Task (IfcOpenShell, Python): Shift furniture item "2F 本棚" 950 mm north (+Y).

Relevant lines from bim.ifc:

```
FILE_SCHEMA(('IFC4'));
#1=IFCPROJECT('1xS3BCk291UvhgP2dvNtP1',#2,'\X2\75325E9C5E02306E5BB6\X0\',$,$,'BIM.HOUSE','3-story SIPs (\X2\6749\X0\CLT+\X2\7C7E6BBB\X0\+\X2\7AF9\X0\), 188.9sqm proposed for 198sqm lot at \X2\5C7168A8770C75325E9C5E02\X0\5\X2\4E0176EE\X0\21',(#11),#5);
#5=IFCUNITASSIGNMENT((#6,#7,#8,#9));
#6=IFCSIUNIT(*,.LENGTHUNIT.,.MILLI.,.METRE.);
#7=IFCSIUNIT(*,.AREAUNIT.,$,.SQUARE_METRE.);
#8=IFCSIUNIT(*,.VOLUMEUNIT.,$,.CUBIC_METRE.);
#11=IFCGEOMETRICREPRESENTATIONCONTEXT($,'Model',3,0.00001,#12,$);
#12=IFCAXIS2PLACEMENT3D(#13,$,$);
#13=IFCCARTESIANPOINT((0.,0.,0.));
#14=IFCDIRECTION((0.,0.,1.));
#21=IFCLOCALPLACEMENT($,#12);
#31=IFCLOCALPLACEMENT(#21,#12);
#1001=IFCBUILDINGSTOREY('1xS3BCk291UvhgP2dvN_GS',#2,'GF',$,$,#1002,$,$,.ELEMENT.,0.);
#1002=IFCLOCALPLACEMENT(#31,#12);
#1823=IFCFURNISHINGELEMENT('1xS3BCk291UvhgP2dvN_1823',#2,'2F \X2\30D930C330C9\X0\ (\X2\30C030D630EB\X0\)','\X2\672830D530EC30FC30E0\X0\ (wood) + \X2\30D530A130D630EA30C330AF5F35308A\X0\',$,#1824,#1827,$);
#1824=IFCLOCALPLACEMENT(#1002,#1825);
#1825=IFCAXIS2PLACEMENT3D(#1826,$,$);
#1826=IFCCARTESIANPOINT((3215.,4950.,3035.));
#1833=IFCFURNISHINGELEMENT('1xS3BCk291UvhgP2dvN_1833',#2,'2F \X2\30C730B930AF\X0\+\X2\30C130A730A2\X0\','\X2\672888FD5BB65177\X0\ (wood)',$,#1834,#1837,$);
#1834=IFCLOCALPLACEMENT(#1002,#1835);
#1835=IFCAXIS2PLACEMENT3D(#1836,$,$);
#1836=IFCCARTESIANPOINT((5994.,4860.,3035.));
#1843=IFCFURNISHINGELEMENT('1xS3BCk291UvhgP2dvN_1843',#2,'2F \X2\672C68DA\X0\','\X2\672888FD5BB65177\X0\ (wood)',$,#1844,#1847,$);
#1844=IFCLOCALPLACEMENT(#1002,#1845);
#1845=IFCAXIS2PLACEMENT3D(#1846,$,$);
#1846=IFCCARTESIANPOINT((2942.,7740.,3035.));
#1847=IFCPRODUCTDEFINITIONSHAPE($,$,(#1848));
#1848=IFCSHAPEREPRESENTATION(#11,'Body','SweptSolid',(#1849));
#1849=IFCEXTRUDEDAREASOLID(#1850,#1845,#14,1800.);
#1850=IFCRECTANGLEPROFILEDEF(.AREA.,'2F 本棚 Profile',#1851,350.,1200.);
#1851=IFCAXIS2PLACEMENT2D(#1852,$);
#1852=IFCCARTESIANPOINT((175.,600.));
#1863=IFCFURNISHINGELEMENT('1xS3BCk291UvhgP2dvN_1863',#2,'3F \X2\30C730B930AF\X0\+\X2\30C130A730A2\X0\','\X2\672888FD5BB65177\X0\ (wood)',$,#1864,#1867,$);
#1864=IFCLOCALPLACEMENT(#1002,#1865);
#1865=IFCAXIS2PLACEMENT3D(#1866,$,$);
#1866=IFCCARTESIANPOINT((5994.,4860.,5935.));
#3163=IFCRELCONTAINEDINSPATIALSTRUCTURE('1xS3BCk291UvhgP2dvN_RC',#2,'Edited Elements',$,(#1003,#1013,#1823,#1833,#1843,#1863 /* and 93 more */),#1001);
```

```python
import ifcopenshell
import ifcopenshell.api.geometry
import ifcopenshell.util.placement
import ifcopenshell.util.unit

model = ifcopenshell.open("bim.ifc")
unit_scale = ifcopenshell.util.unit.calculate_unit_scale(model)

item = model.by_guid("1xS3BCk291UvhgP2dvN_1843")
matrix = ifcopenshell.util.placement.get_local_placement(item.ObjectPlacement)
matrix[1, 3] += 0.95 / unit_scale
ifcopenshell.api.geometry.edit_object_placement(model, product=item, matrix=matrix, is_si=False)

print(ifcopenshell.util.placement.get_local_placement(item.ObjectPlacement).round(3) + 0.0)

model.write("bim_rev.ifc")
```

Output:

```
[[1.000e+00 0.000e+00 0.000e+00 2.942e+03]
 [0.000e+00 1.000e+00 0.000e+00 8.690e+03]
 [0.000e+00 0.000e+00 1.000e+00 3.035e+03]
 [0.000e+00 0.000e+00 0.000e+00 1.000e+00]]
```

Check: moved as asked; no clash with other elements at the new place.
